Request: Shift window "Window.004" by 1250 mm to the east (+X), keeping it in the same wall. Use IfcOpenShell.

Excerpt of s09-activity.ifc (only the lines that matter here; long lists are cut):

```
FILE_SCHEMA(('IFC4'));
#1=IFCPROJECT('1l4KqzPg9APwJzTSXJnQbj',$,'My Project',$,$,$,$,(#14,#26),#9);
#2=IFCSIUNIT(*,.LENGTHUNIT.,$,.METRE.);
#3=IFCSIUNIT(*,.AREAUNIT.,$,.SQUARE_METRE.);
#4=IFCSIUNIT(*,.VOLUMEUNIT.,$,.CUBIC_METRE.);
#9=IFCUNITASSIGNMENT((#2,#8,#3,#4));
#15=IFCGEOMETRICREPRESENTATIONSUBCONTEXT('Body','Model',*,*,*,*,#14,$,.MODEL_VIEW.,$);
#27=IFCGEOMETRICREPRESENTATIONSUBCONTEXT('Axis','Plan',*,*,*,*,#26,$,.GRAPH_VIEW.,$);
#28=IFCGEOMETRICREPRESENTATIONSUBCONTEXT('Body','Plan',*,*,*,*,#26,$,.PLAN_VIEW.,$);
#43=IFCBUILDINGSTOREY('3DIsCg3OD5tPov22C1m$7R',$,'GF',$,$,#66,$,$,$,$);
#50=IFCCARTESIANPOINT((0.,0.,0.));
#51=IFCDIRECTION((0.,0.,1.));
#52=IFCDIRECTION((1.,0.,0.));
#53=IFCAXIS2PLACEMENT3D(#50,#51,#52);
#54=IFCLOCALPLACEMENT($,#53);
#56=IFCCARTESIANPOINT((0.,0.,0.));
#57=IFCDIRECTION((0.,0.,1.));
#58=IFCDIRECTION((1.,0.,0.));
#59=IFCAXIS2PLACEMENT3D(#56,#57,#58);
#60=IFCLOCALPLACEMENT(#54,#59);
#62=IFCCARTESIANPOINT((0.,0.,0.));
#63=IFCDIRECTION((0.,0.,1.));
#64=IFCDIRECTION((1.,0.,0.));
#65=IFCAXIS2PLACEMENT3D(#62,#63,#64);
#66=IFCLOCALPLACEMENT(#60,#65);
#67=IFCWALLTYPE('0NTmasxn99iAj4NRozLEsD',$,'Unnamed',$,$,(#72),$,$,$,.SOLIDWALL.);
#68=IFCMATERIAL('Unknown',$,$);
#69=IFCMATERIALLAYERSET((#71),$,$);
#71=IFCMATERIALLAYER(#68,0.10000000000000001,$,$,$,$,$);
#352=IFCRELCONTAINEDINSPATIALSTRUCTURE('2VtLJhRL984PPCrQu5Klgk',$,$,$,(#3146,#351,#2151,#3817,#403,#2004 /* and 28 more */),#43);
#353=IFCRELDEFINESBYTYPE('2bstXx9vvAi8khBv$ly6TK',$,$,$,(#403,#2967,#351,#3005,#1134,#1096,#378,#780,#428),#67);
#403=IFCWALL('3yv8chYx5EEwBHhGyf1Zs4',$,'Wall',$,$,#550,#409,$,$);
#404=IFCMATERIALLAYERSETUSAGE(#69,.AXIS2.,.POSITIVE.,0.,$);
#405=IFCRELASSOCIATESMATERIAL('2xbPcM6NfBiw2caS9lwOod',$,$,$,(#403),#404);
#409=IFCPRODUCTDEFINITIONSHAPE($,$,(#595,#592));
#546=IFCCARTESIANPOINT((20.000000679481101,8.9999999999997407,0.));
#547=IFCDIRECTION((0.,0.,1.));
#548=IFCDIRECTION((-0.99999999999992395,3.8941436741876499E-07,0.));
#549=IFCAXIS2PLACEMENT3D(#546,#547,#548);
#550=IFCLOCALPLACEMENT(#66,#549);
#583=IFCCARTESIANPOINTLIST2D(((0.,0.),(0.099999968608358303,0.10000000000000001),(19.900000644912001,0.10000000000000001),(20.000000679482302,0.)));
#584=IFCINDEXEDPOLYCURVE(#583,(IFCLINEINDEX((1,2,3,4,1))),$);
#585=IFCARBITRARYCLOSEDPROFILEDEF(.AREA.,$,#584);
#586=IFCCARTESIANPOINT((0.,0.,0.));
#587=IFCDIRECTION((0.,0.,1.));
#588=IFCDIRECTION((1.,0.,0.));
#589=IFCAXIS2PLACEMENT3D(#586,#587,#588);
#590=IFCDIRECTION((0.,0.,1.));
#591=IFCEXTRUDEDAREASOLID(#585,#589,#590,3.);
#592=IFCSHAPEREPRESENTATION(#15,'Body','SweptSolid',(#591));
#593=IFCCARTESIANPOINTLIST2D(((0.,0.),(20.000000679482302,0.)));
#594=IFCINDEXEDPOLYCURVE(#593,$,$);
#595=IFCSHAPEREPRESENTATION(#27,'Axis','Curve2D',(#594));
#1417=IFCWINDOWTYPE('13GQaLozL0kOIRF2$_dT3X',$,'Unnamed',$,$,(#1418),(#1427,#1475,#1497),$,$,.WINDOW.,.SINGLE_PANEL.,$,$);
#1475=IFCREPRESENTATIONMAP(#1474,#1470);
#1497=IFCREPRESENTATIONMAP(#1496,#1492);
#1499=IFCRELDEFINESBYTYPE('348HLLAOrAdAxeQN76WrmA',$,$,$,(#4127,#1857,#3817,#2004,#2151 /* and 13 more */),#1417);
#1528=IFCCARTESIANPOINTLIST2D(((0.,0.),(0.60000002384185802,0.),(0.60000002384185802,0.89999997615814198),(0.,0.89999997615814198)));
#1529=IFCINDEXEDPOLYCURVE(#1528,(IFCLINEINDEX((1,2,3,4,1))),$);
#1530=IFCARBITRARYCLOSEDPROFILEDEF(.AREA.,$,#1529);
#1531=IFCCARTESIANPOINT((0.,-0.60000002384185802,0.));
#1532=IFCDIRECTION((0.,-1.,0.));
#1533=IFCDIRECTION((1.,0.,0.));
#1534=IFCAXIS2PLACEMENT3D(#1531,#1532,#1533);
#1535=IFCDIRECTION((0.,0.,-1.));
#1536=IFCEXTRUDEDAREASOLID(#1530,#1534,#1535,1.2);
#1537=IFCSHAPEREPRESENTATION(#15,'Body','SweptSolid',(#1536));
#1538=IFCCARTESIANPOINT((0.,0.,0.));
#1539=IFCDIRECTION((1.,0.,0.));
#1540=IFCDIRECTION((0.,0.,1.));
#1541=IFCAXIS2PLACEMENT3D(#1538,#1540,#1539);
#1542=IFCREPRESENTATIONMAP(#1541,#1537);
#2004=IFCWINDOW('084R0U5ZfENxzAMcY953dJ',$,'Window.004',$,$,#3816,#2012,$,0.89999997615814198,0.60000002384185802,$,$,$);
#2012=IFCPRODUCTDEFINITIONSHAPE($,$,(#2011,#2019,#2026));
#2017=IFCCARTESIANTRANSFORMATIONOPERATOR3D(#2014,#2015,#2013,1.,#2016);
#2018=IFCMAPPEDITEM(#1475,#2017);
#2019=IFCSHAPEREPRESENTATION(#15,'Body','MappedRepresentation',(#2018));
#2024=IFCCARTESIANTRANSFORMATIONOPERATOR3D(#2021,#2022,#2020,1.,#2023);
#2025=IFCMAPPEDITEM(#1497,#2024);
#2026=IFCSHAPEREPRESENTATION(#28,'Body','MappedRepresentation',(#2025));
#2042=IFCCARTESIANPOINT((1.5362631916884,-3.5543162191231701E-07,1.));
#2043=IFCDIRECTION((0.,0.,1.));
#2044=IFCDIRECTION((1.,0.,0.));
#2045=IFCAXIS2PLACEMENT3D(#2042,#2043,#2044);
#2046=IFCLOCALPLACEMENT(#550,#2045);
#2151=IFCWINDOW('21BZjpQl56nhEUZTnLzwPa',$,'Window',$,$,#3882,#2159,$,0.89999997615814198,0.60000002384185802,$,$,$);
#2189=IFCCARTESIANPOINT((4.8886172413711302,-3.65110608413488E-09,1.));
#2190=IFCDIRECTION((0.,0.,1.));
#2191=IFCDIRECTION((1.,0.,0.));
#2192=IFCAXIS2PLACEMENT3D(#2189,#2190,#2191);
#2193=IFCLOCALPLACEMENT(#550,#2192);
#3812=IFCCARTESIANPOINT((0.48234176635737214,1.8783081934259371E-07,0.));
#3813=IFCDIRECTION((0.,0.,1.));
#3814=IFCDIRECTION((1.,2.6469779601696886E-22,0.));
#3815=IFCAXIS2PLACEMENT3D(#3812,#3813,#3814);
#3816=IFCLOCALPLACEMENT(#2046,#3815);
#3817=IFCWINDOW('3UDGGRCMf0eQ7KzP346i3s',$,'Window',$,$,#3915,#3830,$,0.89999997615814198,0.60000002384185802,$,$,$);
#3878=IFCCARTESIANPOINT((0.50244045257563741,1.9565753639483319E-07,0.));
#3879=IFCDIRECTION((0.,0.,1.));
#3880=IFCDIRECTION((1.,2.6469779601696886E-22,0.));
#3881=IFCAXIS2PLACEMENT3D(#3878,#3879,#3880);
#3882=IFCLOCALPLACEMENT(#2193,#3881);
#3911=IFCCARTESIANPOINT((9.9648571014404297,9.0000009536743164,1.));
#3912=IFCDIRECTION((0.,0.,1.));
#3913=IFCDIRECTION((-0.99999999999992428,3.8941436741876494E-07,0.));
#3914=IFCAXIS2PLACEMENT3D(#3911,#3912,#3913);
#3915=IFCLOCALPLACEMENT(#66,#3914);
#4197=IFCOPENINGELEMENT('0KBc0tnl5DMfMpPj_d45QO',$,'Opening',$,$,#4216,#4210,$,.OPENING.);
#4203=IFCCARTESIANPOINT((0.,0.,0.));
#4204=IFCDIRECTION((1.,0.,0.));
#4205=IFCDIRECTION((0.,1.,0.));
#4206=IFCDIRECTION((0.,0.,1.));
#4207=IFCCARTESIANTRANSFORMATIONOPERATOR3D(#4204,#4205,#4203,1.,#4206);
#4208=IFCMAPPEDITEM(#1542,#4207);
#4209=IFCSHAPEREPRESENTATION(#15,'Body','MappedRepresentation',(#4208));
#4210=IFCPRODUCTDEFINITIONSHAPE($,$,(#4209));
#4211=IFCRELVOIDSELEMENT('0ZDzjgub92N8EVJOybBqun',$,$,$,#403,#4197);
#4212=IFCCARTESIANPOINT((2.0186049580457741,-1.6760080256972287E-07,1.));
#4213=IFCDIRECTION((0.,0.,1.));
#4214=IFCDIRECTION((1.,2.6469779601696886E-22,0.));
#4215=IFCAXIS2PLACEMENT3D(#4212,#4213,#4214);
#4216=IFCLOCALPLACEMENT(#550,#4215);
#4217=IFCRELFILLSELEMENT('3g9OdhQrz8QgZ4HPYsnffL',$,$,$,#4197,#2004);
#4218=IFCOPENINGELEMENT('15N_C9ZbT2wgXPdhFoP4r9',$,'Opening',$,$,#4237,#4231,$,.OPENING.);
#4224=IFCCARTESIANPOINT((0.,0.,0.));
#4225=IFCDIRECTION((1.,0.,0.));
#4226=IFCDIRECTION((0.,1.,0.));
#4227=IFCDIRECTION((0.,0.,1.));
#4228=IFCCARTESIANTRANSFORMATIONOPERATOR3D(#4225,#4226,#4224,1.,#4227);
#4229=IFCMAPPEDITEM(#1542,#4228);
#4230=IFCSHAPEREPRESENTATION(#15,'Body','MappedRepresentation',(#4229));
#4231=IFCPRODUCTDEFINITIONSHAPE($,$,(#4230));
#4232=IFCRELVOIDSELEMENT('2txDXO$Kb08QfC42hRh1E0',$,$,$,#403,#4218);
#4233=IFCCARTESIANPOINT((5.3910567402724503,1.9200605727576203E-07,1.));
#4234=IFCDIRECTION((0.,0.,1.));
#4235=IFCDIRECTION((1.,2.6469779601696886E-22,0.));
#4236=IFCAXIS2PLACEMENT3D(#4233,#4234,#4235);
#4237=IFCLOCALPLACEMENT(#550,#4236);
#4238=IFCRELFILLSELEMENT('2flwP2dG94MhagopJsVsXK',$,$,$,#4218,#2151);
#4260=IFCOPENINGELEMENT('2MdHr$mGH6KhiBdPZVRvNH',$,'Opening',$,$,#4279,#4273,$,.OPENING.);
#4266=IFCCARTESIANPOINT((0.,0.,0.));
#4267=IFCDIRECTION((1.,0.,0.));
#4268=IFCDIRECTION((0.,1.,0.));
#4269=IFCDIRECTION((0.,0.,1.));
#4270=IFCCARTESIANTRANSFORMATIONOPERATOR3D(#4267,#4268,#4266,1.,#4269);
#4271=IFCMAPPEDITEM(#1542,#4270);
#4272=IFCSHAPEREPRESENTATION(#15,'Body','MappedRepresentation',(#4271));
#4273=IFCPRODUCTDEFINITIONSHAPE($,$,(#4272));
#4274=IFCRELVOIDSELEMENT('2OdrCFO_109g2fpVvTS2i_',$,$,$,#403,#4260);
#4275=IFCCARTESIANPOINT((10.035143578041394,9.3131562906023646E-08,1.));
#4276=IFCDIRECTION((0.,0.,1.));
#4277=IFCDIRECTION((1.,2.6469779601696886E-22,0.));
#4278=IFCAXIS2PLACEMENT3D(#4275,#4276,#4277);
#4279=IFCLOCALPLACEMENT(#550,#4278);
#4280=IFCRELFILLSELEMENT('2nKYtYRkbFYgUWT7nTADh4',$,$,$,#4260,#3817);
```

```python
import ifcopenshell
import ifcopenshell.api.geometry
import ifcopenshell.util.placement
import ifcopenshell.util.unit

model = ifcopenshell.open("s09-activity.ifc")
unit_scale = ifcopenshell.util.unit.calculate_unit_scale(model)

window = model.by_guid("084R0U5ZfENxzAMcY953dJ")
opening = window.FillsVoids[0].RelatingOpeningElement
wall = opening.VoidsElements[0].RelatingBuildingElement

wall_matrix = ifcopenshell.util.placement.get_local_placement(wall.ObjectPlacement)
shift = wall_matrix[:3, 0] * -1.25 / unit_scale
before = ifcopenshell.util.placement.get_local_placement(window.ObjectPlacement)[:3, 3].copy()

# The window is not placed relative to its opening, so move both.
for product in (opening, window):
    matrix = ifcopenshell.util.placement.get_local_placement(product.ObjectPlacement)
    matrix[:3, 3] += shift
    ifcopenshell.api.geometry.edit_object_placement(model, product=product, matrix=matrix, is_si=False)

after = ifcopenshell.util.placement.get_local_placement(window.ObjectPlacement)[:3, 3]
print("window moved by", (after - before).round(3) + 0.0)

model.write("s09-activity_updated.ifc")
```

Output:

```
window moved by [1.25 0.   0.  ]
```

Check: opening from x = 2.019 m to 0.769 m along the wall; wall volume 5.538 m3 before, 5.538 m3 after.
